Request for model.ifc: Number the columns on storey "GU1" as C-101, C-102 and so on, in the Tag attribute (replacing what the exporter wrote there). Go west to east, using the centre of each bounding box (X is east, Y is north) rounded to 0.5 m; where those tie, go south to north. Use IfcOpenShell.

First a look at what the model holds.

```python
import ifcopenshell
import ifcopenshell.util.element
import ifcopenshell.util.placement

model = ifcopenshell.open("model.ifc")
print(model.schema)
storey = next(s for s in model.by_type("IfcBuildingStorey") if s.Name == "GU1")
columns = [e for e in ifcopenshell.util.element.get_decomposition(storey) if e.is_a("IfcColumn")]
for e in sorted(columns, key=lambda e: e.id()):
    origin = ifcopenshell.util.placement.get_local_placement(e.ObjectPlacement)[:3, 3]
    print(e.id(), e.Tag, e.Name, origin.round(2) + 0.0, sep=" | ")
```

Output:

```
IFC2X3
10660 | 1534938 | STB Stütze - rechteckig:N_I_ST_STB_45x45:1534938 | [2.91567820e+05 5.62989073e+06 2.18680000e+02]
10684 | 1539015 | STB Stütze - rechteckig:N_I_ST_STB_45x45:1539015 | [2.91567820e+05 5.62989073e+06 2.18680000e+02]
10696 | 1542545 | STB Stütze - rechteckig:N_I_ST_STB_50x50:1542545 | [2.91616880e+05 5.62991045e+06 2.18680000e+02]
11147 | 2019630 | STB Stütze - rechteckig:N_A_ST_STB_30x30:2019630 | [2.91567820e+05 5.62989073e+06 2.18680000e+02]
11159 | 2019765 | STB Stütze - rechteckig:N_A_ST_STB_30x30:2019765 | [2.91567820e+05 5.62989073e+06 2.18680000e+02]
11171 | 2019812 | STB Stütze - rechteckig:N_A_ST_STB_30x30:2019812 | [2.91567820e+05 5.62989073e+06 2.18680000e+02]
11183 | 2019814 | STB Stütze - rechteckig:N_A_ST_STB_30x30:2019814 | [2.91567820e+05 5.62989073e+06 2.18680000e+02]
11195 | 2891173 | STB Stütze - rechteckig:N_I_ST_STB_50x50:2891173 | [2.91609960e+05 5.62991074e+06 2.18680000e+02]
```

```python
import ifcopenshell
import ifcopenshell.geom
import ifcopenshell.util.element
import ifcopenshell.util.shape

model = ifcopenshell.open("model.ifc")
settings = ifcopenshell.geom.settings()
settings.set("use-world-coords", True)


def centre(element):
    shape = ifcopenshell.geom.create_shape(settings, element)
    return ifcopenshell.util.shape.get_bbox_centroid(shape.geometry)


storey = next(s for s in model.by_type("IfcBuildingStorey") if s.Name == "GU1")
columns = [e for e in ifcopenshell.util.element.get_decomposition(storey) if e.is_a("IfcColumn")]

# Insertion points can sit at a corner or the storey origin, so sort by the geometry (in metres).
centres = {e: centre(e) for e in columns}
columns.sort(key=lambda e: (round(centres[e][0] / 0.5), centres[e][1]))

for i, e in enumerate(columns, start=1):
    number = f"C-1{i:02d}"
    e.Tag = number
    print(e.id(), number)

model.write("model-out.ifc")
```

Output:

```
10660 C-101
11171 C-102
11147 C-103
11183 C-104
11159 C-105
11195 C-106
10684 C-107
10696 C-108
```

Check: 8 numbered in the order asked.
